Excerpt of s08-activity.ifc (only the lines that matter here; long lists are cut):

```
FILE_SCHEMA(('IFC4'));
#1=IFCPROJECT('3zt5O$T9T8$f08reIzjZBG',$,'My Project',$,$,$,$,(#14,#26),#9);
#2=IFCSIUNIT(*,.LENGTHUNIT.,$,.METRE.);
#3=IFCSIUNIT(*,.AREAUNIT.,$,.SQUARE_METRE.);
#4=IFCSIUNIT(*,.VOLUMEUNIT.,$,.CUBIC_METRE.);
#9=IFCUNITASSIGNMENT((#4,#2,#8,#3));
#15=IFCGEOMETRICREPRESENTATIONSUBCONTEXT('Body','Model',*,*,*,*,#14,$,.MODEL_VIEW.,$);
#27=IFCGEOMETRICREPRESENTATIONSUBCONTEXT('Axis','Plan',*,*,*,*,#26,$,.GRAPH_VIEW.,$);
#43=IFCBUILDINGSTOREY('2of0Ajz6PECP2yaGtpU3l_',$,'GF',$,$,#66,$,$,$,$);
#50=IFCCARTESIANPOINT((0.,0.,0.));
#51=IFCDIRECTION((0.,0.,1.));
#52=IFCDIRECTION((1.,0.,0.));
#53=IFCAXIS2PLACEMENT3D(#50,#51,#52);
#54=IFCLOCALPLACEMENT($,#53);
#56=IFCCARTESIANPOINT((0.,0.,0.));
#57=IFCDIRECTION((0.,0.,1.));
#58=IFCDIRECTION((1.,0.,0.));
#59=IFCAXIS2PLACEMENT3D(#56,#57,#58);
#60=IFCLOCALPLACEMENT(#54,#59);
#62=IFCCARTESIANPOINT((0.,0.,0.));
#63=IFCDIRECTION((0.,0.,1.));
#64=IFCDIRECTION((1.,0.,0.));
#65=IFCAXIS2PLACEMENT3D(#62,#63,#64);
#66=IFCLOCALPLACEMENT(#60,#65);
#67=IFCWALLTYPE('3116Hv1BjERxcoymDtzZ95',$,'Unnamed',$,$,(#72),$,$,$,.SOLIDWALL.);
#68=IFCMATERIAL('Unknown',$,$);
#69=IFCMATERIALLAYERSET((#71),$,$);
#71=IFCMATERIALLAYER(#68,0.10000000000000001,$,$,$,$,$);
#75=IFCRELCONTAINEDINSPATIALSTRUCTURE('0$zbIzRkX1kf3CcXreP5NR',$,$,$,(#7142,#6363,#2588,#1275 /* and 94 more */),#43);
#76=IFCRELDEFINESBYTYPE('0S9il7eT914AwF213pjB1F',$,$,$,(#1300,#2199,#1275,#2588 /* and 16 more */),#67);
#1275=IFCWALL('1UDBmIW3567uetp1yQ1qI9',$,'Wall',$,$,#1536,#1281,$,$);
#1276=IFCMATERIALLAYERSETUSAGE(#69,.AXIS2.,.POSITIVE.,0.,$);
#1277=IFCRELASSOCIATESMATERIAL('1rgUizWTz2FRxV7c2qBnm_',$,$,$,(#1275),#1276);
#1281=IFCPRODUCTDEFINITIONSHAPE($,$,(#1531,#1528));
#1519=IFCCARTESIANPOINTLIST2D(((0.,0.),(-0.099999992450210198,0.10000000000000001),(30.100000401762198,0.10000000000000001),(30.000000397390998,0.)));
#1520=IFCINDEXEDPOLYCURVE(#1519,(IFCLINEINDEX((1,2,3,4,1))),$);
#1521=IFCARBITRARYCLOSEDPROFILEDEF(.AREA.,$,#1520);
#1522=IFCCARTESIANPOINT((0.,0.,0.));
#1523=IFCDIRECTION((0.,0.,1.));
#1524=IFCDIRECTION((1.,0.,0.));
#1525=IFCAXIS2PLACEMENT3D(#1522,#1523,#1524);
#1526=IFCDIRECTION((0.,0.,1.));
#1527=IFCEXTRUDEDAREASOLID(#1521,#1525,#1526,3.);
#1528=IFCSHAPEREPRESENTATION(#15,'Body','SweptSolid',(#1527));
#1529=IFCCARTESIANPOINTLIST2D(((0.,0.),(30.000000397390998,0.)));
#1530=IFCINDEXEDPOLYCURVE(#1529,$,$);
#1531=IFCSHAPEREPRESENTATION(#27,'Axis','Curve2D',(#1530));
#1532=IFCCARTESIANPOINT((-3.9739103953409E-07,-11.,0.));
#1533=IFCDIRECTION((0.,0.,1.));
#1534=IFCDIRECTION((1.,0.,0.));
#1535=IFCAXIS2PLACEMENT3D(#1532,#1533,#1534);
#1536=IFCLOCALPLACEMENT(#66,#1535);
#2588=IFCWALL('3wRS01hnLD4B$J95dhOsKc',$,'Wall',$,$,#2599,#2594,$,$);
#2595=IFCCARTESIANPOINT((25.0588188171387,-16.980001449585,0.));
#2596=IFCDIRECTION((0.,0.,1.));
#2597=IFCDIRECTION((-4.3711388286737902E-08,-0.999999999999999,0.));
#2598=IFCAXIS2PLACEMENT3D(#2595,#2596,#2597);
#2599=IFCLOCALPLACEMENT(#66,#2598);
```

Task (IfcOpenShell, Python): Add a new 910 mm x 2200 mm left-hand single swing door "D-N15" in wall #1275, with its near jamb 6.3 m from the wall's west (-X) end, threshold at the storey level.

```python
import numpy as np
import ifcopenshell
import ifcopenshell.api.feature
import ifcopenshell.api.geometry
import ifcopenshell.api.root
import ifcopenshell.api.spatial
import ifcopenshell.geom
import ifcopenshell.util.element
import ifcopenshell.util.placement
import ifcopenshell.util.representation
import ifcopenshell.util.shape
import ifcopenshell.util.unit

model = ifcopenshell.open("s08-activity.ifc")
unit_scale = ifcopenshell.util.unit.calculate_unit_scale(model)
settings = ifcopenshell.geom.settings()


def volume(element):
    """Net volume in cubic metres, openings subtracted."""
    shape = ifcopenshell.geom.create_shape(settings, element)
    return ifcopenshell.util.shape.get_volume(shape.geometry)


wall = model.by_id(1275)
storey = ifcopenshell.util.element.get_container(wall, ifc_class="IfcBuildingStorey")
context = ifcopenshell.util.representation.get_context(model, "Model", "Body", "MODEL_VIEW")
before = volume(wall)

width, height, from_end, sill = 0.91, 2.2, 6.3, 0.0  # metres

# The wall runs along its own X axis, and the end named is its -X end.
wall_shape = ifcopenshell.geom.create_shape(settings, wall)
x, y, z = ifcopenshell.util.shape.get_vertices(wall_shape.geometry).T
start = x.min() + from_end
face, thickness = float(y.min()), float(y.max() - y.min())
wall_matrix = ifcopenshell.util.placement.get_local_placement(wall.ObjectPlacement)
level = ifcopenshell.util.placement.get_local_placement(storey.ObjectPlacement)[2, 3]


def in_wall(x, y):
    """Placement at x, y metres in the wall's axes, at sill height."""
    matrix = wall_matrix.copy()
    matrix[:, 3] = wall_matrix @ np.array([x / unit_scale, y / unit_scale, 0.0, 1.0])
    matrix[2, 3] = level + sill / unit_scale
    return matrix


# Opening: a box that overshoots both wall faces by 50 mm.
opening = ifcopenshell.api.root.create_entity(model, ifc_class="IfcOpeningElement", predefined_type="OPENING")
box = ifcopenshell.api.geometry.add_wall_representation(
    model, context=context, length=width, height=height, thickness=thickness + 0.1
)
ifcopenshell.api.geometry.assign_representation(model, product=opening, representation=box)
ifcopenshell.api.geometry.edit_object_placement(model, product=opening, matrix=in_wall(start, face - 0.05), is_si=False)
ifcopenshell.api.feature.add_feature(model, feature=opening, element=wall)

door = ifcopenshell.api.root.create_entity(model, ifc_class="IfcDoor", name="D-N15", predefined_type="DOOR")
door.OverallWidth, door.OverallHeight = width / unit_scale, height / unit_scale
door.OperationType = "SINGLE_SWING_LEFT"
body = ifcopenshell.api.geometry.add_door_representation(
    model,
    context=context,
    overall_width=door.OverallWidth,
    overall_height=door.OverallHeight,
    operation_type="SINGLE_SWING_LEFT",
    lining_properties={"LiningDepth": thickness / unit_scale, "ThresholdDepth": thickness / unit_scale},
)
ifcopenshell.api.geometry.assign_representation(model, product=door, representation=body)
ifcopenshell.api.spatial.assign_container(model, products=[door], relating_structure=storey)
ifcopenshell.api.feature.add_filling(model, opening=opening, element=door)

# The lining spans the wall, so the door starts at the wall face.
ifcopenshell.api.geometry.edit_object_placement(model, product=door, matrix=in_wall(start, face), is_si=False)

after = volume(wall)

print(f"wall volume {before:.3f} -> {after:.3f} m3")

model.write("s08-activity_v2.ifc")
```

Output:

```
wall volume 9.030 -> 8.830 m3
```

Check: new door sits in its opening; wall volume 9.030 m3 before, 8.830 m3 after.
